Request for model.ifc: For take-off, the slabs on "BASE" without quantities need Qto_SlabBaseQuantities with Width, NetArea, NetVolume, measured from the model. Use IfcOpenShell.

First a look at what the model holds.

```python
import ifcopenshell
import ifcopenshell.util.element
import ifcopenshell.util.unit

model = ifcopenshell.open("model.ifc")
print(model.schema)
for unit_type in ("LENGTHUNIT", "AREAUNIT", "VOLUMEUNIT"):
    print(unit_type, ifcopenshell.util.unit.calculate_unit_scale(model, unit_type))
storey = next(s for s in model.by_type("IfcBuildingStorey") if s.Name == "BASE")
slabs = [e for e in ifcopenshell.util.element.get_decomposition(storey) if e.is_a("IfcSlab")]
for e in sorted(slabs, key=lambda e: e.id()):
    print(e.id(), e.is_a(), e.Name, list(ifcopenshell.util.element.get_psets(e, qtos_only=True)), sep=" | ")
```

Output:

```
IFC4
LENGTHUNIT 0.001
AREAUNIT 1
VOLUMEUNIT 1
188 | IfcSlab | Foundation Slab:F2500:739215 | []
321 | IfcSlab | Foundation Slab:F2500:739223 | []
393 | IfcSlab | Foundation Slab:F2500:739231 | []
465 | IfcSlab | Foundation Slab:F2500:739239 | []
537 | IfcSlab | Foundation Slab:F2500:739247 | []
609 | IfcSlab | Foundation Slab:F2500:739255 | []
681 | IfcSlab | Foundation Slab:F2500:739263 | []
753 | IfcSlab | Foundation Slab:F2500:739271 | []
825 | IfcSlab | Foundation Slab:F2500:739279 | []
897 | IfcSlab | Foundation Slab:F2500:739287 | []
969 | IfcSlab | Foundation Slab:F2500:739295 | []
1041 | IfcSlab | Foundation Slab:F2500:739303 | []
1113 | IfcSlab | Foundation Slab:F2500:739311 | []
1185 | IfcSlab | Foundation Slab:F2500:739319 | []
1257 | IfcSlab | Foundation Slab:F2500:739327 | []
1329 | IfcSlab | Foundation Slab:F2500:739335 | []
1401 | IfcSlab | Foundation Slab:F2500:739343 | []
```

```python
import ifcopenshell
import ifcopenshell.api.pset
import ifcopenshell.geom
import ifcopenshell.util.element
import ifcopenshell.util.shape
import ifcopenshell.util.unit

model = ifcopenshell.open("model.ifc")
unit_scale = ifcopenshell.util.unit.calculate_unit_scale(model)
area_scale = ifcopenshell.util.unit.calculate_unit_scale(model, "AREAUNIT")
volume_scale = ifcopenshell.util.unit.calculate_unit_scale(model, "VOLUMEUNIT")
settings = ifcopenshell.geom.settings()

storey = next(s for s in model.by_type("IfcBuildingStorey") if s.Name == "BASE")
slabs = [e for e in ifcopenshell.util.element.get_decomposition(storey) if e.is_a("IfcSlab")]

for e in sorted(slabs, key=lambda e: e.id()):
    if ifcopenshell.util.element.get_psets(e, qtos_only=True, should_inherit=False):
        continue
    # Geometry comes back in metres, in the element's own axes.
    shape = ifcopenshell.geom.create_shape(settings, e)
    values = {
        "Width": ifcopenshell.util.shape.get_z(shape.geometry) / unit_scale,
        "NetArea": ifcopenshell.util.shape.get_footprint_area(shape.geometry) / area_scale,
        "NetVolume": ifcopenshell.util.shape.get_volume(shape.geometry) / volume_scale,
    }
    qto = ifcopenshell.api.pset.add_qto(model, product=e, name="Qto_SlabBaseQuantities")
    ifcopenshell.api.pset.edit_qto(model, qto=qto, properties=values)
    print(e.id(), {k: round(v, 3) for k, v in values.items()})

model.write("model_edited.ifc")
```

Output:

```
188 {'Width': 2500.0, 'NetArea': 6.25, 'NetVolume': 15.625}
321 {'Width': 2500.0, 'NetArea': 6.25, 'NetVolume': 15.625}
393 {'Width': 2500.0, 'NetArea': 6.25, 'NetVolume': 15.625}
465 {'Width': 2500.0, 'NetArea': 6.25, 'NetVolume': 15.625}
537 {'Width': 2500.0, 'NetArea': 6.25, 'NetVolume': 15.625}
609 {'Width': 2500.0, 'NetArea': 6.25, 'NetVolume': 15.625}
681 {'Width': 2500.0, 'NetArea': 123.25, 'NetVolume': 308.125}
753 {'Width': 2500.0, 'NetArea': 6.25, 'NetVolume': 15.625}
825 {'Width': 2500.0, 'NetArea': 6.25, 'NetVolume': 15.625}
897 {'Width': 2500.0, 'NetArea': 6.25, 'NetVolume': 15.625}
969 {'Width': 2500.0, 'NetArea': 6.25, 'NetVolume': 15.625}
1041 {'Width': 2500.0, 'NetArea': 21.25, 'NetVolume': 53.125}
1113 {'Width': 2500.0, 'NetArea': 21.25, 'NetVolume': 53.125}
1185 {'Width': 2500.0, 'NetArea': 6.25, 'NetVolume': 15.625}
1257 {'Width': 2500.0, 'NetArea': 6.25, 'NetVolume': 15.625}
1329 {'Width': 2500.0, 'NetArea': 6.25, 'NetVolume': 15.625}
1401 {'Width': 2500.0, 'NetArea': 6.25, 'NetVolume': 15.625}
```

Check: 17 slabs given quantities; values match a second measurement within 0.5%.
